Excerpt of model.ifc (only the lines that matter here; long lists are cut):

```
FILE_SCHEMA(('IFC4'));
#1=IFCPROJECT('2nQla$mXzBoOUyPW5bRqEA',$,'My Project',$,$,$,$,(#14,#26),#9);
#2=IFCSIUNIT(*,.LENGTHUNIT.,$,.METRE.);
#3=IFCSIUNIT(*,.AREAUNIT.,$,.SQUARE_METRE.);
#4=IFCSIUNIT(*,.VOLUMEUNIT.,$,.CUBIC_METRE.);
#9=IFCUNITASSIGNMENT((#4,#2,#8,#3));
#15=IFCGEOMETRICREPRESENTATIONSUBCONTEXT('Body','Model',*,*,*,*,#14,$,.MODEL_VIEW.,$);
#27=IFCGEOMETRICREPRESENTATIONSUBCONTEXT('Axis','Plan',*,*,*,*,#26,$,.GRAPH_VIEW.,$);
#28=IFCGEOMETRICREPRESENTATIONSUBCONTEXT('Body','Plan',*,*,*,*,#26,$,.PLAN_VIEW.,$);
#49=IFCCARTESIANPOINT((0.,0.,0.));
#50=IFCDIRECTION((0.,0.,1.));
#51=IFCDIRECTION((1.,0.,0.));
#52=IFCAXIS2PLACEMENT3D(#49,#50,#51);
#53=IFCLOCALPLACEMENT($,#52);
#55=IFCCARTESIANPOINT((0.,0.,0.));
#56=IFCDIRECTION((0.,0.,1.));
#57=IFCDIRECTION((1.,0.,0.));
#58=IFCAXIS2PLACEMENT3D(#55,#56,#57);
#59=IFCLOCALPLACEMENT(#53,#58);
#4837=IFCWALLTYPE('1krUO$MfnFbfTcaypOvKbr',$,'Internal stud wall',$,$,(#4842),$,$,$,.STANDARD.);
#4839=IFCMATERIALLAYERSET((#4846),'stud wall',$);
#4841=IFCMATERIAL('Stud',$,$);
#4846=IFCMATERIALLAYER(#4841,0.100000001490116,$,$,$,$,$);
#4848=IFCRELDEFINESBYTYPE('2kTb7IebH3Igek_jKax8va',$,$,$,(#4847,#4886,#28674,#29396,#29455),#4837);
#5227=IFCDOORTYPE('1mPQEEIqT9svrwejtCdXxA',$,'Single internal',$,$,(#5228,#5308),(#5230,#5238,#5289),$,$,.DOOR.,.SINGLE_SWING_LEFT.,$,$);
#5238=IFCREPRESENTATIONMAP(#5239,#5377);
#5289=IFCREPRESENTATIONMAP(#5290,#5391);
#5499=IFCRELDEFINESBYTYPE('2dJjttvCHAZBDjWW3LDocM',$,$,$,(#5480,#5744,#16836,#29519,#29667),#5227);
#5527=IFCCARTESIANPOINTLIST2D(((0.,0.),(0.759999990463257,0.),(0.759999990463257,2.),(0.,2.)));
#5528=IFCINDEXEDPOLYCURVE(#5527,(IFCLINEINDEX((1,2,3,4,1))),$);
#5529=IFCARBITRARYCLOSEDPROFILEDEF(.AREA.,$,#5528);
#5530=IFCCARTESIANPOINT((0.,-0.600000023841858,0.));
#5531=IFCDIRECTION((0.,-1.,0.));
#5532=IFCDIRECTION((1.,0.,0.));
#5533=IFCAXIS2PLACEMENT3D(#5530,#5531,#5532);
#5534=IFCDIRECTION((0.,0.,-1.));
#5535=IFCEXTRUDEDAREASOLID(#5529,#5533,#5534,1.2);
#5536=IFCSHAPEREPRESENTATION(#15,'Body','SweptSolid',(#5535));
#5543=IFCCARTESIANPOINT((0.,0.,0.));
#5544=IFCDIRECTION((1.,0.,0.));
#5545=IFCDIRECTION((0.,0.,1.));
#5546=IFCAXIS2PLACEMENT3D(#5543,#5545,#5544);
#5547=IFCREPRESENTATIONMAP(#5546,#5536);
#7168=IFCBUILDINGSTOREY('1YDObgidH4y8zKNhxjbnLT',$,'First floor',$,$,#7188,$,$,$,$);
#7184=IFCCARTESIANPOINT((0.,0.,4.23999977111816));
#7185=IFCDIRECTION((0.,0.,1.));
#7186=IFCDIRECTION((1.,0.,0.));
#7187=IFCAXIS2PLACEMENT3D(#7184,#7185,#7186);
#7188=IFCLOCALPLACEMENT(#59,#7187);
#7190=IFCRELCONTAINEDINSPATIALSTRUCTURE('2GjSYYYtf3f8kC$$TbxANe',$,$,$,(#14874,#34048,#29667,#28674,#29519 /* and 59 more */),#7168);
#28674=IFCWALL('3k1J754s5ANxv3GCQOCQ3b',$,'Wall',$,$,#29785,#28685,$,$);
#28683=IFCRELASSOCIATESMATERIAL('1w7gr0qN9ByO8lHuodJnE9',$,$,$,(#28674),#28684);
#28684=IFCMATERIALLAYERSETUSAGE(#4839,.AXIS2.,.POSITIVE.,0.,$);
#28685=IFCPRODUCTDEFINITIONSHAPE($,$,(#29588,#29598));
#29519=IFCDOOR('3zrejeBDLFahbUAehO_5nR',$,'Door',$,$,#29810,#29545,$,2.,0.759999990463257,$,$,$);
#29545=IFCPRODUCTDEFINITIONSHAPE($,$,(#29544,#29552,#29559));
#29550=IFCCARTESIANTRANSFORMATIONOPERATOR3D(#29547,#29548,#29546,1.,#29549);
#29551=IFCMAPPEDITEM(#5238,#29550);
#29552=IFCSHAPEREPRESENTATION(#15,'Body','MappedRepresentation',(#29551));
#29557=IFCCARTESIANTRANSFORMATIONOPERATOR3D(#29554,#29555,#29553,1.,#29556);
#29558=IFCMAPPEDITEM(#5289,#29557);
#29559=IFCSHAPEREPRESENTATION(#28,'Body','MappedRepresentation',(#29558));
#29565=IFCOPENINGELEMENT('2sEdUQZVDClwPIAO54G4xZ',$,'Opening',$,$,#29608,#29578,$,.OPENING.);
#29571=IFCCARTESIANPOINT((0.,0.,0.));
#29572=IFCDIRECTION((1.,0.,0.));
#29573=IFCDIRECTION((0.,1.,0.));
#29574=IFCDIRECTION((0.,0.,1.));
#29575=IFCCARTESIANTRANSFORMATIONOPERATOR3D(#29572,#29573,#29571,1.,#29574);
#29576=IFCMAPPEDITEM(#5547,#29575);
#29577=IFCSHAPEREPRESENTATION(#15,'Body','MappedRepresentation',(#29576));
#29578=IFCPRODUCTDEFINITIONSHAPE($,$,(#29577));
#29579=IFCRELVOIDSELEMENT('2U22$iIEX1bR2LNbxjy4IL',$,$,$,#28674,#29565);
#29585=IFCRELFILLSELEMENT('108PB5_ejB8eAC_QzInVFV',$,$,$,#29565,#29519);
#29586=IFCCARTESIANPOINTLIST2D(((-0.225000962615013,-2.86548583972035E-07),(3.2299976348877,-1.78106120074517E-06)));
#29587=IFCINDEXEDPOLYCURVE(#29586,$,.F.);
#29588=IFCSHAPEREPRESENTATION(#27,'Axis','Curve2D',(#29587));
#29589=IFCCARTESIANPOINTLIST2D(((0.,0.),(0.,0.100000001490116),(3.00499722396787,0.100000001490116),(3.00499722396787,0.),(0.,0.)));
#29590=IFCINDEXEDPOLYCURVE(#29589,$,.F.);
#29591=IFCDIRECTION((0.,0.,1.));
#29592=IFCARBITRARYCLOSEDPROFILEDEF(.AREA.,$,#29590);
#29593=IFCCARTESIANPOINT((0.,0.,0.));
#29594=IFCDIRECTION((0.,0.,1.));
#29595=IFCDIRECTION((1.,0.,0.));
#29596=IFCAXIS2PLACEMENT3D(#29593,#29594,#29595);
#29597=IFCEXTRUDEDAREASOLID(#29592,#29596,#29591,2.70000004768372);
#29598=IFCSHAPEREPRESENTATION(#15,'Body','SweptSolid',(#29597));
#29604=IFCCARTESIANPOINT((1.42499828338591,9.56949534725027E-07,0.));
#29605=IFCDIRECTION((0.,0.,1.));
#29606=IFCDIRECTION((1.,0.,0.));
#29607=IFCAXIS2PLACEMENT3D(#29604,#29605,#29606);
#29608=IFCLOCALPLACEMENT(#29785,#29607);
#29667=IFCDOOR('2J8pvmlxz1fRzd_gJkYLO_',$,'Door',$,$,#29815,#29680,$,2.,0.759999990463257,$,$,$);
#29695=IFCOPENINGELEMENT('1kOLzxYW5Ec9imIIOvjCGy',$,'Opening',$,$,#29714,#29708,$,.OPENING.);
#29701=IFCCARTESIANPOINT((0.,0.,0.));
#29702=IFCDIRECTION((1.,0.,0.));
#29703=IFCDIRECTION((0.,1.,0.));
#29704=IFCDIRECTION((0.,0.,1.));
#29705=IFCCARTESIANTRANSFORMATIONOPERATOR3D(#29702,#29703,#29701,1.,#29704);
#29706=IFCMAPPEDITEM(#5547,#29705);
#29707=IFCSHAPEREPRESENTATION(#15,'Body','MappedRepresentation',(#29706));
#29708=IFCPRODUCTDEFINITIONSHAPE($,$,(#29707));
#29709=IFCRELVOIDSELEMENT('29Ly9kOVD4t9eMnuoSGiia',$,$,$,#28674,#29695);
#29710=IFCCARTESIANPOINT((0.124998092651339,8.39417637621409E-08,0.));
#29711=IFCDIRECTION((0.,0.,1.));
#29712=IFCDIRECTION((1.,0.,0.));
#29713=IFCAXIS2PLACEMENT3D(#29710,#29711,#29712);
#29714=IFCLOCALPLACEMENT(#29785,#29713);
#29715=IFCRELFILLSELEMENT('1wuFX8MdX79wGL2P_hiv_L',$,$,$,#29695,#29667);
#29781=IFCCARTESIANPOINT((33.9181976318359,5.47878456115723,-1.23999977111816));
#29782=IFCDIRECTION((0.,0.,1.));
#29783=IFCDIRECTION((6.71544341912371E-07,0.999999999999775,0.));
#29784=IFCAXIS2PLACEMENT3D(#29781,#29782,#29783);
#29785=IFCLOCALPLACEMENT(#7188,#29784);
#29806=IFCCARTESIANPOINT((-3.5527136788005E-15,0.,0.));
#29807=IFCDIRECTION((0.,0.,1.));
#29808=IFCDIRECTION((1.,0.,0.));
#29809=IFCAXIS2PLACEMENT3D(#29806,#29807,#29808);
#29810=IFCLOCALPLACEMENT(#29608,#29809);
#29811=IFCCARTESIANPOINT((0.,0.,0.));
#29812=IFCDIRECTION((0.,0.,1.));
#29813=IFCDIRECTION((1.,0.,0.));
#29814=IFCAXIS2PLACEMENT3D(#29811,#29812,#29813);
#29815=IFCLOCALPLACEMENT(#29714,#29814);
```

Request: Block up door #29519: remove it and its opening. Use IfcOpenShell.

```python
import ifcopenshell
import ifcopenshell.api.feature
import ifcopenshell.api.root
import ifcopenshell.geom
import ifcopenshell.util.shape

model = ifcopenshell.open("model.ifc")
settings = ifcopenshell.geom.settings()


def volume(element):
    """Net volume in cubic metres, openings subtracted."""
    shape = ifcopenshell.geom.create_shape(settings, element)
    return ifcopenshell.util.shape.get_volume(shape.geometry)


door = model.by_guid("3zrejeBDLFahbUAehO_5nR")
opening = door.FillsVoids[0].RelatingOpeningElement
wall = opening.VoidsElements[0].RelatingBuildingElement
before = volume(wall)

ifcopenshell.api.root.remove_product(model, product=door)
ifcopenshell.api.feature.remove_feature(model, feature=opening)

after = volume(wall)

print(f"wall volume {before:.3f} -> {after:.3f} m3")

model.write("model_rev.ifc")
```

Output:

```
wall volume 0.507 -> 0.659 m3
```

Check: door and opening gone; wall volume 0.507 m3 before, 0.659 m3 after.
